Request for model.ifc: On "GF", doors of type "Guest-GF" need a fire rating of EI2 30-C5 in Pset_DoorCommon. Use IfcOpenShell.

First a look at what the model holds.

```python
import ifcopenshell
import ifcopenshell.util.element

model = ifcopenshell.open("model.ifc")
print(model.schema)
storey = next(s for s in model.by_type("IfcBuildingStorey") if s.Name == "GF")
doors = [e for e in ifcopenshell.util.element.get_decomposition(storey) if e.is_a("IfcDoor")]
seen = {}
for e in doors:
    element_type = ifcopenshell.util.element.get_type(e)
    key = (element_type.Name if element_type != e and element_type else None, ifcopenshell.util.element.get_pset(e, "Pset_DoorCommon", "FireRating"))
    seen[key] = seen.get(key, 0) + 1
for (name, value), count in sorted(seen.items(), key=str):
    print(count, "x", name, "|", value)
```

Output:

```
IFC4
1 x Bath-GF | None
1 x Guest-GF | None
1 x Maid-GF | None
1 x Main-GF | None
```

```python
import ifcopenshell
import ifcopenshell.api.pset
import ifcopenshell.util.element

model = ifcopenshell.open("model.ifc")

storey = next(s for s in model.by_type("IfcBuildingStorey") if s.Name == "GF")
doors = [e for e in ifcopenshell.util.element.get_decomposition(storey) if e.is_a("IfcDoor")]

count = 0
for e in doors:
    element_type = ifcopenshell.util.element.get_type(e)
    if element_type in (None, e) or element_type.Name != "Guest-GF":
        continue
    # add_pset returns the element's existing set when there is one.
    pset = ifcopenshell.api.pset.add_pset(model, product=e, name="Pset_DoorCommon")
    ifcopenshell.api.pset.edit_pset(model, pset=pset, properties={"FireRating": "EI2 30-C5"})
    count += 1

print(count, "doors updated")

model.write("model_v2.ifc")
```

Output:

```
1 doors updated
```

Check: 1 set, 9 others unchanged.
